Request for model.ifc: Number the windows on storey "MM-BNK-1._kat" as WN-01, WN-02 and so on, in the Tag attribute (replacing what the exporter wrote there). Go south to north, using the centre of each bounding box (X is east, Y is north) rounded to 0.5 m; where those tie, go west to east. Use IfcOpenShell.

First a look at what the model holds.

```python
import ifcopenshell
import ifcopenshell.util.element
import ifcopenshell.util.placement

model = ifcopenshell.open("model.ifc")
print(model.schema)
storey = next(s for s in model.by_type("IfcBuildingStorey") if s.Name == "MM-BNK-1._kat")
windows = [e for e in ifcopenshell.util.element.get_decomposition(storey) if e.is_a("IfcWindow")]
for e in sorted(windows, key=lambda e: e.id()):
    origin = ifcopenshell.util.placement.get_local_placement(e.ObjectPlacement)[:3, 3]
    print(e.id(), e.Tag, e.Name, origin.round(2) + 0.0, sep=" | ")
```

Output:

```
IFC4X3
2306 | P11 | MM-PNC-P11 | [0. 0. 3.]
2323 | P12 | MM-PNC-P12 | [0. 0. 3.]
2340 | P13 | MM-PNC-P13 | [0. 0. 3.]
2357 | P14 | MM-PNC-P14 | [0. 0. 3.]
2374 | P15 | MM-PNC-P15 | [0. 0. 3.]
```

```python
import ifcopenshell
import ifcopenshell.geom
import ifcopenshell.util.element
import ifcopenshell.util.shape

model = ifcopenshell.open("model.ifc")
settings = ifcopenshell.geom.settings()
settings.set("use-world-coords", True)


def centre(element):
    shape = ifcopenshell.geom.create_shape(settings, element)
    return ifcopenshell.util.shape.get_bbox_centroid(shape.geometry)


storey = next(s for s in model.by_type("IfcBuildingStorey") if s.Name == "MM-BNK-1._kat")
windows = [e for e in ifcopenshell.util.element.get_decomposition(storey) if e.is_a("IfcWindow")]

# Insertion points can sit at a corner or the storey origin, so sort by the geometry (in metres).
centres = {e: centre(e) for e in windows}
windows.sort(key=lambda e: (round(centres[e][1] / 0.5), centres[e][0]))

for i, e in enumerate(windows, start=1):
    number = f"WN-{i:02d}"
    e.Tag = number
    print(e.id(), number)

model.write("model_edited.ifc")
```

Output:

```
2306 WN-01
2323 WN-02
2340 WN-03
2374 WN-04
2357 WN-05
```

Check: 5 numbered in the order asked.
